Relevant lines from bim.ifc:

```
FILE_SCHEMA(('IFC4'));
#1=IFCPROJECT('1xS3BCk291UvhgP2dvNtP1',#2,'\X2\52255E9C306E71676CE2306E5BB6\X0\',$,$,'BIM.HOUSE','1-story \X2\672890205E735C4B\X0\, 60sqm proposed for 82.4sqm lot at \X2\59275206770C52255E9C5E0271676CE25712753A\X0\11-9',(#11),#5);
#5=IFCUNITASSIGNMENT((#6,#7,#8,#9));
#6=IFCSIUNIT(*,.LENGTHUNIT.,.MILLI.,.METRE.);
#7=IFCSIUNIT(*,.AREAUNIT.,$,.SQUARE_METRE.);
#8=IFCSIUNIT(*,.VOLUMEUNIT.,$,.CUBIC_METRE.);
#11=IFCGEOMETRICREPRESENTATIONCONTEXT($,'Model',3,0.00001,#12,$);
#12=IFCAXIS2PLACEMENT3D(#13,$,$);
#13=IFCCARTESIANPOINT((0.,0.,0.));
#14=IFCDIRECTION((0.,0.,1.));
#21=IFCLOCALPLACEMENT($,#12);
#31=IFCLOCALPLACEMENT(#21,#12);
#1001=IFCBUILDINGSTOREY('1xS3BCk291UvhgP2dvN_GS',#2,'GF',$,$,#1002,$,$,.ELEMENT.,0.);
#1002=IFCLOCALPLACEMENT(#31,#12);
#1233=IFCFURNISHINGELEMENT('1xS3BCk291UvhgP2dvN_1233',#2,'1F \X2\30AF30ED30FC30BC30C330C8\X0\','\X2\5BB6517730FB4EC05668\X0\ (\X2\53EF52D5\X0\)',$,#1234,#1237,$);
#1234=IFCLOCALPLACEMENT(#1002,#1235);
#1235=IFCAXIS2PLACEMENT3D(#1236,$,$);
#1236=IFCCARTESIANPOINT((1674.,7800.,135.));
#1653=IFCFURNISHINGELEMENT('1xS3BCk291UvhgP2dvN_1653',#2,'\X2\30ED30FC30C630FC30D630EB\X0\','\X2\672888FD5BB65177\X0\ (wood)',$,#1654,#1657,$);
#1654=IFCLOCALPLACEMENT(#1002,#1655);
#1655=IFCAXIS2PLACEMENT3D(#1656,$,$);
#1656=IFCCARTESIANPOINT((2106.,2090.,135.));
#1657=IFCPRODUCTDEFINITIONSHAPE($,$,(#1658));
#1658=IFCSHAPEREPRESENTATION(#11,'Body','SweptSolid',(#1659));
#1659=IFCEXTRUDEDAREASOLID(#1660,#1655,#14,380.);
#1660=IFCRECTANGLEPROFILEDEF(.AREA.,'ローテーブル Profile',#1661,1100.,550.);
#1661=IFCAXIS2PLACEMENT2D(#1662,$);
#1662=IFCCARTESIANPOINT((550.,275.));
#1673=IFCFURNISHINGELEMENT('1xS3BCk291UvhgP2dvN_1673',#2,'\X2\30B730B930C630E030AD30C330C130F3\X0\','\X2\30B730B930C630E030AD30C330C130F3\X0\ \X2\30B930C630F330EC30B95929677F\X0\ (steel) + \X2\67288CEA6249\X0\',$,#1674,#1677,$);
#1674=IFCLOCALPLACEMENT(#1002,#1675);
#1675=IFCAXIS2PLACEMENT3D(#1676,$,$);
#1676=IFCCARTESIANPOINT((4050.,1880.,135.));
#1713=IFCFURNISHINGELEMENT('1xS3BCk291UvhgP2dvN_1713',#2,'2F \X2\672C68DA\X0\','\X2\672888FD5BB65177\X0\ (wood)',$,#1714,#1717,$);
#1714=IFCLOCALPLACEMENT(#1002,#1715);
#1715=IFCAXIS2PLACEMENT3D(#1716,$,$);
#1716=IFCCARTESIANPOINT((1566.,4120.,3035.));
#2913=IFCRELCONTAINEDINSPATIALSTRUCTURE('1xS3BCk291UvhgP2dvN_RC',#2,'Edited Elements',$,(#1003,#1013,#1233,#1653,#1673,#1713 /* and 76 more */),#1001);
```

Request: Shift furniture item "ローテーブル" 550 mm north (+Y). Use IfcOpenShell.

```python
import ifcopenshell
import ifcopenshell.api.geometry
import ifcopenshell.util.placement

model = ifcopenshell.open("bim.ifc")

item = model.by_guid("1xS3BCk291UvhgP2dvN_1653")
matrix = ifcopenshell.util.placement.get_local_placement(item.ObjectPlacement)
matrix[1, 3] += 550.0
ifcopenshell.api.geometry.edit_object_placement(model, product=item, matrix=matrix, is_si=False)

print(ifcopenshell.util.placement.get_local_placement(item.ObjectPlacement).round(3) + 0.0)

model.write("bim_v2.ifc")
```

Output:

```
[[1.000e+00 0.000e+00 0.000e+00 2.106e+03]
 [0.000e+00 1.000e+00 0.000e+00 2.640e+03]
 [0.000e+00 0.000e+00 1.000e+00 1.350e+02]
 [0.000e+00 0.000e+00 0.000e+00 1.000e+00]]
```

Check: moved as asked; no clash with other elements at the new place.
